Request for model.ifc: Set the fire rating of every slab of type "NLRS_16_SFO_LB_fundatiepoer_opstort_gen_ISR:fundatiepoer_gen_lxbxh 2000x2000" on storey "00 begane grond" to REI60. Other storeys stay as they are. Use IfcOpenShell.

First a look at what the model holds.

```python
import ifcopenshell
import ifcopenshell.util.element

model = ifcopenshell.open("model.ifc")
print(model.schema)
storey = next(s for s in model.by_type("IfcBuildingStorey") if s.Name == "00 begane grond")
slabs = [e for e in ifcopenshell.util.element.get_decomposition(storey) if e.is_a("IfcSlab")]
seen = {}
for e in slabs:
    element_type = ifcopenshell.util.element.get_type(e)
    key = (element_type.Name if element_type != e and element_type else None, ifcopenshell.util.element.get_pset(e, "Pset_SlabCommon", "FireRating"))
    seen[key] = seen.get(key, 0) + 1
for (name, value), count in sorted(seen.items(), key=str):
    print(count, "x", name, "|", value)
```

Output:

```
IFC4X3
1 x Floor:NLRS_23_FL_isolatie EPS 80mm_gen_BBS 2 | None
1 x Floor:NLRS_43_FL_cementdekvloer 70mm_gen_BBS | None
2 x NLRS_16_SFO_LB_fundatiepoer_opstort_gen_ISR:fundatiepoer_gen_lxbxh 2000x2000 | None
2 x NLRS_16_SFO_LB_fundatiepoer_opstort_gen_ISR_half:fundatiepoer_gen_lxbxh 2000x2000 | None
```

```python
import ifcopenshell
import ifcopenshell.api.pset
import ifcopenshell.util.element

model = ifcopenshell.open("model.ifc")

storey = next(s for s in model.by_type("IfcBuildingStorey") if s.Name == "00 begane grond")
slabs = [e for e in ifcopenshell.util.element.get_decomposition(storey) if e.is_a("IfcSlab")]

count = 0
for e in slabs:
    element_type = ifcopenshell.util.element.get_type(e)
    if element_type in (None, e) or element_type.Name != "NLRS_16_SFO_LB_fundatiepoer_opstort_gen_ISR:fundatiepoer_gen_lxbxh 2000x2000":
        continue
    # add_pset returns the element's existing set when there is one.
    pset = ifcopenshell.api.pset.add_pset(model, product=e, name="Pset_SlabCommon")
    ifcopenshell.api.pset.edit_pset(model, pset=pset, properties={"FireRating": "REI60"})
    count += 1

print(count, "slabs updated")

model.write("model_v2.ifc")
```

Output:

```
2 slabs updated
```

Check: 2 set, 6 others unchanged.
